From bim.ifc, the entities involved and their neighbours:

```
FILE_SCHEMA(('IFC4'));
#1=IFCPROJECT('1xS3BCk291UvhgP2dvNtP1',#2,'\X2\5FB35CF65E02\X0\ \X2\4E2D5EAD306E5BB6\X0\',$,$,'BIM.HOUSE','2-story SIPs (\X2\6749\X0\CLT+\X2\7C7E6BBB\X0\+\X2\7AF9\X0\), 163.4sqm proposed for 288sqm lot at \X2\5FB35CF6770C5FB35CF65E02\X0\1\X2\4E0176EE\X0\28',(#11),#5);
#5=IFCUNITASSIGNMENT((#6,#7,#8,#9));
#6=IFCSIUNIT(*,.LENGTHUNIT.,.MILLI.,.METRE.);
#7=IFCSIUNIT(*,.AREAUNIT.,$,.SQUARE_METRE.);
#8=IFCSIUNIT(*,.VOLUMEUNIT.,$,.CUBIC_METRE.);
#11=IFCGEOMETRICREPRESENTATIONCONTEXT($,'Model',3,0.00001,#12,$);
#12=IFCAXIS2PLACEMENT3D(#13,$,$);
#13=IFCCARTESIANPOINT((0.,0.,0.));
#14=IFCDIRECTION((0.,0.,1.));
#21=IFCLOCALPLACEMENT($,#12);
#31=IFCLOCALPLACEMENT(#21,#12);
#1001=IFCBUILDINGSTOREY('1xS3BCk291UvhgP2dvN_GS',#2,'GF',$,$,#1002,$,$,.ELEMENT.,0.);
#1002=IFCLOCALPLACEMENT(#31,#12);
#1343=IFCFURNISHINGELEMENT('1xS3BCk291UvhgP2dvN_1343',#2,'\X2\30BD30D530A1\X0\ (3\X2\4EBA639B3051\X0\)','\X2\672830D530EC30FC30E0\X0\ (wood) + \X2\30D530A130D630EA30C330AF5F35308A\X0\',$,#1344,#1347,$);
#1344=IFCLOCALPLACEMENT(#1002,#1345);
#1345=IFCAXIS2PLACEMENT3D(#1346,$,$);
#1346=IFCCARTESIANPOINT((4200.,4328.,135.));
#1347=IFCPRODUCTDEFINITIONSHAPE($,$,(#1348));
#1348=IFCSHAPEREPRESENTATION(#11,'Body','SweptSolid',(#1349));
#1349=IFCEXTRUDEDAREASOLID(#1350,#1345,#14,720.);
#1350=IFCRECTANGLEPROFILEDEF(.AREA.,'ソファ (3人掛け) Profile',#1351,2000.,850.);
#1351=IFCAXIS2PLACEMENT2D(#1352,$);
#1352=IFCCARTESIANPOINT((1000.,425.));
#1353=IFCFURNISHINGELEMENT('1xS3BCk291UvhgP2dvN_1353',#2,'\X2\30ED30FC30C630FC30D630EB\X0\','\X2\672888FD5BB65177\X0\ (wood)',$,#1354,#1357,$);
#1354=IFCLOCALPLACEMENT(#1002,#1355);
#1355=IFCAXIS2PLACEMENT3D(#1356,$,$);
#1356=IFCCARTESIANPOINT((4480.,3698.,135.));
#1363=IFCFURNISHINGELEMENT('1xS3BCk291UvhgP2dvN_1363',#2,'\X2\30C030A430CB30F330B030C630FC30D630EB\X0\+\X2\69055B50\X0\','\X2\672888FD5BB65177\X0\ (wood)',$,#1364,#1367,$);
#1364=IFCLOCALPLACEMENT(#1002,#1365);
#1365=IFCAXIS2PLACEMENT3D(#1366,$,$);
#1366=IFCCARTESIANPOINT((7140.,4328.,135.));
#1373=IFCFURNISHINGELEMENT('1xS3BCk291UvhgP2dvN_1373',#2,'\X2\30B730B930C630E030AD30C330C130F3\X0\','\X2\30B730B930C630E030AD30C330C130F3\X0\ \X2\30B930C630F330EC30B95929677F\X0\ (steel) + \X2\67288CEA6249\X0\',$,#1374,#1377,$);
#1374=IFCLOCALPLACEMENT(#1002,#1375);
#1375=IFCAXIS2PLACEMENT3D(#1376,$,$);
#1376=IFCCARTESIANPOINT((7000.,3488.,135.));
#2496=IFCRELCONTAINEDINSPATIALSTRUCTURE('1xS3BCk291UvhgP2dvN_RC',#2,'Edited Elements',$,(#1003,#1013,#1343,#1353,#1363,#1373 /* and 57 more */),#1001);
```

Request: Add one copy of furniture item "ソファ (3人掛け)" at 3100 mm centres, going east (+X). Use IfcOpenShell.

```python
import numpy as np
import ifcopenshell
import ifcopenshell.api.geometry
import ifcopenshell.api.root
import ifcopenshell.util.element
import ifcopenshell.util.placement

model = ifcopenshell.open("bim.ifc")


def reuse_history(source, copy):
    """copy_class also copies each property set's owner history, people and application; keep the originals."""
    for rel in copy.IsDefinedBy:
        if rel.is_a("IfcRelDefinesByProperties") and (history := rel.RelatingPropertyDefinition.OwnerHistory):
            rel.RelatingPropertyDefinition.OwnerHistory = source.OwnerHistory
            ifcopenshell.util.element.remove_deep2(model, history)


source = model.by_id(1343)
base = ifcopenshell.util.placement.get_local_placement(source.ObjectPlacement)
step = np.array([1.0, 0.0, 0.0]) * 3100.0

for i in range(1, 2):
    copy = ifcopenshell.api.root.copy_class(model, product=source)
    copy.Representation = ifcopenshell.util.element.copy_deep(
        model, source.Representation, exclude=["IfcGeometricRepresentationContext", "IfcRepresentationMap"]
    )
    reuse_history(source, copy)
    matrix = base.copy()
    matrix[:3, 3] += i * step
    print("added at", matrix[:3, 3].round(3) + 0.0)
    ifcopenshell.api.geometry.edit_object_placement(model, product=copy, matrix=matrix, is_si=False)

model.write("bim_rev.ifc")
```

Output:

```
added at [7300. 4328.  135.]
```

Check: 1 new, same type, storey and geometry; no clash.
